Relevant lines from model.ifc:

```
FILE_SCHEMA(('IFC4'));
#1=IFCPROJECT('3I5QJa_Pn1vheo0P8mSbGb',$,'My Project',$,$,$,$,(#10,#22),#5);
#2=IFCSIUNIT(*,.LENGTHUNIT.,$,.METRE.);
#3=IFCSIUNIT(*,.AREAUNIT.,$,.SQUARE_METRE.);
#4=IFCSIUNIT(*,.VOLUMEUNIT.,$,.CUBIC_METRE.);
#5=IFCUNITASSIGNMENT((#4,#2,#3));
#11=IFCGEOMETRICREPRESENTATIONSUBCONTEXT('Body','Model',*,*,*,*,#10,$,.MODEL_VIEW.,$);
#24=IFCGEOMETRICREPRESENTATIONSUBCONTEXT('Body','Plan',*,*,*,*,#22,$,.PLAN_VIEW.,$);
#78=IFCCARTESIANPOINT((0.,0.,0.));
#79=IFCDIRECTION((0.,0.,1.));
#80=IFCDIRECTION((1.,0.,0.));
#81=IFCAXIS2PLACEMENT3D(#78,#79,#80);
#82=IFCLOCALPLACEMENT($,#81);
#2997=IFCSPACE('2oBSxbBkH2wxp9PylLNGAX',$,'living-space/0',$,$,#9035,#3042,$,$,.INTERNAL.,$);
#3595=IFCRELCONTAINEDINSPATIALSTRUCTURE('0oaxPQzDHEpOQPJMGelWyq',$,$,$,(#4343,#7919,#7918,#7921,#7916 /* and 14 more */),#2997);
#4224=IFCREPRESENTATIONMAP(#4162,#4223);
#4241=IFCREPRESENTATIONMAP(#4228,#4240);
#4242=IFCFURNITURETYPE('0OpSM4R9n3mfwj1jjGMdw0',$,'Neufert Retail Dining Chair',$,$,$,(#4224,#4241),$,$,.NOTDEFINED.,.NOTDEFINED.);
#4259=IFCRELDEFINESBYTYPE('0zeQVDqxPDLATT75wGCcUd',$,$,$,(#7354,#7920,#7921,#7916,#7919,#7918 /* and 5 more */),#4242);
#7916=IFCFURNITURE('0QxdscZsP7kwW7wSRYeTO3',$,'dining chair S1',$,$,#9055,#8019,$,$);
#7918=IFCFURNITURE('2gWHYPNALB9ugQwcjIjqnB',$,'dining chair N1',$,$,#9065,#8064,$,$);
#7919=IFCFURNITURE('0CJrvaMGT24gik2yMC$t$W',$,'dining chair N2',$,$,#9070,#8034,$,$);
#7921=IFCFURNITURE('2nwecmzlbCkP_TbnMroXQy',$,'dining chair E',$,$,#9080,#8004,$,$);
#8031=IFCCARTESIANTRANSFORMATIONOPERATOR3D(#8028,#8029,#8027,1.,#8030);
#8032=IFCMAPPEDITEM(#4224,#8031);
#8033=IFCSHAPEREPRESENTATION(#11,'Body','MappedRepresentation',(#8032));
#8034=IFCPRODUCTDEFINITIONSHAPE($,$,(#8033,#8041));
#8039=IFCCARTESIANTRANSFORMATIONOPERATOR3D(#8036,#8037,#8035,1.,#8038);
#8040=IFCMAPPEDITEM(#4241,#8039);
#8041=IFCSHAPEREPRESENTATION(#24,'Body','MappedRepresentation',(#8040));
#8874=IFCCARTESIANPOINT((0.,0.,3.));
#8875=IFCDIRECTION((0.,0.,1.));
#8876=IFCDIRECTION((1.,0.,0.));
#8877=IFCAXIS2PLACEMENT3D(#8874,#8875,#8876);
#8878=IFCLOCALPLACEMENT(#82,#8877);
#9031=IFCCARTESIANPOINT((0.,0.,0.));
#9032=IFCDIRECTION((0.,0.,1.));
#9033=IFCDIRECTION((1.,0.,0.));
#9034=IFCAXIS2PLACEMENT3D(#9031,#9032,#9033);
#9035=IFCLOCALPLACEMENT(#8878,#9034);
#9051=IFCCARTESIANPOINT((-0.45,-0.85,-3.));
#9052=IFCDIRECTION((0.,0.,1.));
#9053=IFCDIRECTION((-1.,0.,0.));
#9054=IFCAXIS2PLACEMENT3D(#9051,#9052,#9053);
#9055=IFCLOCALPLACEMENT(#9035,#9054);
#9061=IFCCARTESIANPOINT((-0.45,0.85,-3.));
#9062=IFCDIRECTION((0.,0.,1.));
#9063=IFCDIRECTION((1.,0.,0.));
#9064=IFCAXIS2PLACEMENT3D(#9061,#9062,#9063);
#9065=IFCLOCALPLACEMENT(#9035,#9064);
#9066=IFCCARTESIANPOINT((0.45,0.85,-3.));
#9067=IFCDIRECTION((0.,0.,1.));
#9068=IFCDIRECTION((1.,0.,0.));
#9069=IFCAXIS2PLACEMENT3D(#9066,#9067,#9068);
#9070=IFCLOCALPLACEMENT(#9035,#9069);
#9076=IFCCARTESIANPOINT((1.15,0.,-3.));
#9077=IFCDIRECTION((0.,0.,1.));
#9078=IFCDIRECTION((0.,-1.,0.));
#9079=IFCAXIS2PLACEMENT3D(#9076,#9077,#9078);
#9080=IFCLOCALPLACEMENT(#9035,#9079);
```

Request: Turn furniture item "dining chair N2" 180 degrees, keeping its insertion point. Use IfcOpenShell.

```python
import ifcopenshell
import ifcopenshell.api.geometry
import ifcopenshell.util.placement

model = ifcopenshell.open("model.ifc")

item = model.by_guid("0CJrvaMGT24gik2yMC$t$W")
matrix = ifcopenshell.util.placement.get_local_placement(item.ObjectPlacement)
matrix = matrix @ ifcopenshell.util.placement.rotation(180, "Z")
ifcopenshell.api.geometry.edit_object_placement(model, product=item, matrix=matrix, is_si=False)

print(ifcopenshell.util.placement.get_local_placement(item.ObjectPlacement).round(3) + 0.0)

model.write("model_edited.ifc")
```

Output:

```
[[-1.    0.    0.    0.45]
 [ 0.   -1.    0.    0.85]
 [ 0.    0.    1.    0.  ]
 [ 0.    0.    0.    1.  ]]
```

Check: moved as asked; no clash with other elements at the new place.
